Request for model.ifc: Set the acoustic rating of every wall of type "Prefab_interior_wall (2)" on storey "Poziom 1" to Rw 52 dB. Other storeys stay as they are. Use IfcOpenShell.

First a look at what the model holds.

```python
import ifcopenshell
import ifcopenshell.util.element

model = ifcopenshell.open("model.ifc")
print(model.schema)
storey = next(s for s in model.by_type("IfcBuildingStorey") if s.Name == "Poziom 1")
walls = [e for e in ifcopenshell.util.element.get_decomposition(storey) if e.is_a("IfcWall")]
seen = {}
for e in walls:
    element_type = ifcopenshell.util.element.get_type(e)
    key = (element_type.Name if element_type != e and element_type else None, ifcopenshell.util.element.get_pset(e, "Pset_WallCommon", "AcousticRating"))
    seen[key] = seen.get(key, 0) + 1
for (name, value), count in sorted(seen.items(), key=str):
    print(count, "x", name, "|", value)
```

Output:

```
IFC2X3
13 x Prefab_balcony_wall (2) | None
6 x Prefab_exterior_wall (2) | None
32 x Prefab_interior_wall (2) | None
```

```python
import ifcopenshell
import ifcopenshell.api.pset
import ifcopenshell.util.element

model = ifcopenshell.open("model.ifc")

storey = next(s for s in model.by_type("IfcBuildingStorey") if s.Name == "Poziom 1")
walls = [e for e in ifcopenshell.util.element.get_decomposition(storey) if e.is_a("IfcWall")]

count = 0
for e in walls:
    element_type = ifcopenshell.util.element.get_type(e)
    if element_type in (None, e) or element_type.Name != "Prefab_interior_wall (2)":
        continue
    # add_pset returns the element's existing set when there is one.
    pset = ifcopenshell.api.pset.add_pset(model, product=e, name="Pset_WallCommon")
    ifcopenshell.api.pset.edit_pset(model, pset=pset, properties={"AcousticRating": "Rw 52 dB"})
    count += 1

print(count, "walls updated")

model.write("model_v2.ifc")
```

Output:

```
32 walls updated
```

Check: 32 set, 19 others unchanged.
